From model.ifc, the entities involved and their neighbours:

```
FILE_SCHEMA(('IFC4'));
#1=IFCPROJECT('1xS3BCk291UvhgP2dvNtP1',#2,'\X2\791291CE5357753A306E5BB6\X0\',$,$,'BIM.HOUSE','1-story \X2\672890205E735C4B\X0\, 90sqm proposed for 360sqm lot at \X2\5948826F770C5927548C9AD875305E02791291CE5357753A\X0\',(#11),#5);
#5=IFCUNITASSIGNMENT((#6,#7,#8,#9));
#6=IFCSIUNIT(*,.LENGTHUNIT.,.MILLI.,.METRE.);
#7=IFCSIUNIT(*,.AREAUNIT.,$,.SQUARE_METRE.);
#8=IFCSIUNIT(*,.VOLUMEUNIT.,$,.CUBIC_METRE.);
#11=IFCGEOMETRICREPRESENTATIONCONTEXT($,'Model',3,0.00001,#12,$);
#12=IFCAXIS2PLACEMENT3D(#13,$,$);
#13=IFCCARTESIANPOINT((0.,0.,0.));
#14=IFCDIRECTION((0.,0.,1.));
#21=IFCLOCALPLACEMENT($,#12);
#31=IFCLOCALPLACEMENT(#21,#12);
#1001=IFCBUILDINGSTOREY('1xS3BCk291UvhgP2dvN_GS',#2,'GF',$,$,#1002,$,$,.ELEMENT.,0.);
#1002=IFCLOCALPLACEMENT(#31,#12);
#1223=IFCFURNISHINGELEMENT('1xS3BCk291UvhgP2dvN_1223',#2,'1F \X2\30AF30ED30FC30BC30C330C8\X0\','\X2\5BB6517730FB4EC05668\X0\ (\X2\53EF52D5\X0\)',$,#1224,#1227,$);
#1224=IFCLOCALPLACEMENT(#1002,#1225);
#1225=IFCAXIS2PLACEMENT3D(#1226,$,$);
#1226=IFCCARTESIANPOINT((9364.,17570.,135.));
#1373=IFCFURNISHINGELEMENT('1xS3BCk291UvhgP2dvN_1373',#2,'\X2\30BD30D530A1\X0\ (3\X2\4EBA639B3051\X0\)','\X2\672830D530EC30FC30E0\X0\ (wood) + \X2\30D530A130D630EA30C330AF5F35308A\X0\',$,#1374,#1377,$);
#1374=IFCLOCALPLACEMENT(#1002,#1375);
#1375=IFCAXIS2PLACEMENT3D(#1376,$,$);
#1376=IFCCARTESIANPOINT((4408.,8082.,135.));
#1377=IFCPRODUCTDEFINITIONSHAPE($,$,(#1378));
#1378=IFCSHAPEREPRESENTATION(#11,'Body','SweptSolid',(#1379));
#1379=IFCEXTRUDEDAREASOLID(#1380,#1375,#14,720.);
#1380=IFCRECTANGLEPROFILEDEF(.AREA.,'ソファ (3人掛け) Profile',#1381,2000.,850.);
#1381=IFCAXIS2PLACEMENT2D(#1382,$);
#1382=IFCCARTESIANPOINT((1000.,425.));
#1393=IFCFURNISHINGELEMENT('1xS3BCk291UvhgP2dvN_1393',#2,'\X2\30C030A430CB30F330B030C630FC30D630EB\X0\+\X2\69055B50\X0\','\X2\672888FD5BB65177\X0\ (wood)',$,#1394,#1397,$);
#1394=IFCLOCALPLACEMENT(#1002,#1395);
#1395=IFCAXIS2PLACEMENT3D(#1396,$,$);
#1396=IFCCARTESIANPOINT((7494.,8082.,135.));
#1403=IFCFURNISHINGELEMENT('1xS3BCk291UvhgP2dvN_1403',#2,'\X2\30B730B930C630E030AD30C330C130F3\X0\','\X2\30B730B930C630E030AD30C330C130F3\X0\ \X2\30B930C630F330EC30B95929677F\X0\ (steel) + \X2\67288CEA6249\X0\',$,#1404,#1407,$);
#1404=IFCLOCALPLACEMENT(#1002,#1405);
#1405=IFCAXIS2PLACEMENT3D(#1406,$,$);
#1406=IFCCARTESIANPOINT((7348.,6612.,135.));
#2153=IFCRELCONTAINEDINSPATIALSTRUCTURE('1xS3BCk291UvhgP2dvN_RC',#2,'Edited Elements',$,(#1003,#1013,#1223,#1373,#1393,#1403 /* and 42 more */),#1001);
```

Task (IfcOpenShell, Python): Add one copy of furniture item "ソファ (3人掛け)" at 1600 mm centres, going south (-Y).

```python
import numpy as np
import ifcopenshell
import ifcopenshell.api.geometry
import ifcopenshell.api.root
import ifcopenshell.util.element
import ifcopenshell.util.placement
import ifcopenshell.util.unit

model = ifcopenshell.open("model.ifc")
unit_scale = ifcopenshell.util.unit.calculate_unit_scale(model)


def reuse_history(source, copy):
    """copy_class also copies each property set's owner history, people and application; keep the originals."""
    for rel in copy.IsDefinedBy:
        if rel.is_a("IfcRelDefinesByProperties") and (history := rel.RelatingPropertyDefinition.OwnerHistory):
            rel.RelatingPropertyDefinition.OwnerHistory = source.OwnerHistory
            ifcopenshell.util.element.remove_deep2(model, history)


source = model.by_guid("1xS3BCk291UvhgP2dvN_1373")
base = ifcopenshell.util.placement.get_local_placement(source.ObjectPlacement)
step = np.array([0.0, -1.0, 0.0]) * 1.6 / unit_scale

for i in range(1, 2):
    copy = ifcopenshell.api.root.copy_class(model, product=source)
    copy.Representation = ifcopenshell.util.element.copy_deep(
        model, source.Representation, exclude=["IfcGeometricRepresentationContext", "IfcRepresentationMap"]
    )
    reuse_history(source, copy)
    matrix = base.copy()
    matrix[:3, 3] += i * step
    print("added at", matrix[:3, 3].round(3) + 0.0)
    ifcopenshell.api.geometry.edit_object_placement(model, product=copy, matrix=matrix, is_si=False)

model.write("model_v2.ifc")
```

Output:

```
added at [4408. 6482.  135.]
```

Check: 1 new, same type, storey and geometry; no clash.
